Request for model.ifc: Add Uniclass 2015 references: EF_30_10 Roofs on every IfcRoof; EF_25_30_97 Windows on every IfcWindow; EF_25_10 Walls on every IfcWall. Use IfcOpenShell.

First a look at what the model holds.

```python
import ifcopenshell

model = ifcopenshell.open("model.ifc")
print(model.schema)
print("classifications:", [c.Name for c in model.by_type("IfcClassification")])
for ifc_class in ("IfcDoor", "IfcRoof", "IfcStair", "IfcWall", "IfcWindow"):
    print(ifc_class, len(model.by_type(ifc_class)))
```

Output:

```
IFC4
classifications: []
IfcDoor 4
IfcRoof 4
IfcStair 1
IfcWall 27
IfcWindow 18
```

```python
import ifcopenshell
import ifcopenshell.api.classification

model = ifcopenshell.open("model.ifc")

system = ifcopenshell.api.classification.add_classification(model, classification="Uniclass 2015")

codes = {
    "IfcRoof": ("EF_30_10", "Roofs"),
    "IfcWindow": ("EF_25_30_97", "Windows"),
    "IfcWall": ("EF_25_10", "Walls"),
}
for ifc_class, (code, name) in codes.items():
    products = model.by_type(ifc_class)
    ifcopenshell.api.classification.add_reference(
        model, products=products, classification=system, identification=code, name=name
    )
    print(code, len(products))

model.write("model_rev.ifc")
```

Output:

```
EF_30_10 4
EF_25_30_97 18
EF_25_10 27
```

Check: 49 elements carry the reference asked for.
